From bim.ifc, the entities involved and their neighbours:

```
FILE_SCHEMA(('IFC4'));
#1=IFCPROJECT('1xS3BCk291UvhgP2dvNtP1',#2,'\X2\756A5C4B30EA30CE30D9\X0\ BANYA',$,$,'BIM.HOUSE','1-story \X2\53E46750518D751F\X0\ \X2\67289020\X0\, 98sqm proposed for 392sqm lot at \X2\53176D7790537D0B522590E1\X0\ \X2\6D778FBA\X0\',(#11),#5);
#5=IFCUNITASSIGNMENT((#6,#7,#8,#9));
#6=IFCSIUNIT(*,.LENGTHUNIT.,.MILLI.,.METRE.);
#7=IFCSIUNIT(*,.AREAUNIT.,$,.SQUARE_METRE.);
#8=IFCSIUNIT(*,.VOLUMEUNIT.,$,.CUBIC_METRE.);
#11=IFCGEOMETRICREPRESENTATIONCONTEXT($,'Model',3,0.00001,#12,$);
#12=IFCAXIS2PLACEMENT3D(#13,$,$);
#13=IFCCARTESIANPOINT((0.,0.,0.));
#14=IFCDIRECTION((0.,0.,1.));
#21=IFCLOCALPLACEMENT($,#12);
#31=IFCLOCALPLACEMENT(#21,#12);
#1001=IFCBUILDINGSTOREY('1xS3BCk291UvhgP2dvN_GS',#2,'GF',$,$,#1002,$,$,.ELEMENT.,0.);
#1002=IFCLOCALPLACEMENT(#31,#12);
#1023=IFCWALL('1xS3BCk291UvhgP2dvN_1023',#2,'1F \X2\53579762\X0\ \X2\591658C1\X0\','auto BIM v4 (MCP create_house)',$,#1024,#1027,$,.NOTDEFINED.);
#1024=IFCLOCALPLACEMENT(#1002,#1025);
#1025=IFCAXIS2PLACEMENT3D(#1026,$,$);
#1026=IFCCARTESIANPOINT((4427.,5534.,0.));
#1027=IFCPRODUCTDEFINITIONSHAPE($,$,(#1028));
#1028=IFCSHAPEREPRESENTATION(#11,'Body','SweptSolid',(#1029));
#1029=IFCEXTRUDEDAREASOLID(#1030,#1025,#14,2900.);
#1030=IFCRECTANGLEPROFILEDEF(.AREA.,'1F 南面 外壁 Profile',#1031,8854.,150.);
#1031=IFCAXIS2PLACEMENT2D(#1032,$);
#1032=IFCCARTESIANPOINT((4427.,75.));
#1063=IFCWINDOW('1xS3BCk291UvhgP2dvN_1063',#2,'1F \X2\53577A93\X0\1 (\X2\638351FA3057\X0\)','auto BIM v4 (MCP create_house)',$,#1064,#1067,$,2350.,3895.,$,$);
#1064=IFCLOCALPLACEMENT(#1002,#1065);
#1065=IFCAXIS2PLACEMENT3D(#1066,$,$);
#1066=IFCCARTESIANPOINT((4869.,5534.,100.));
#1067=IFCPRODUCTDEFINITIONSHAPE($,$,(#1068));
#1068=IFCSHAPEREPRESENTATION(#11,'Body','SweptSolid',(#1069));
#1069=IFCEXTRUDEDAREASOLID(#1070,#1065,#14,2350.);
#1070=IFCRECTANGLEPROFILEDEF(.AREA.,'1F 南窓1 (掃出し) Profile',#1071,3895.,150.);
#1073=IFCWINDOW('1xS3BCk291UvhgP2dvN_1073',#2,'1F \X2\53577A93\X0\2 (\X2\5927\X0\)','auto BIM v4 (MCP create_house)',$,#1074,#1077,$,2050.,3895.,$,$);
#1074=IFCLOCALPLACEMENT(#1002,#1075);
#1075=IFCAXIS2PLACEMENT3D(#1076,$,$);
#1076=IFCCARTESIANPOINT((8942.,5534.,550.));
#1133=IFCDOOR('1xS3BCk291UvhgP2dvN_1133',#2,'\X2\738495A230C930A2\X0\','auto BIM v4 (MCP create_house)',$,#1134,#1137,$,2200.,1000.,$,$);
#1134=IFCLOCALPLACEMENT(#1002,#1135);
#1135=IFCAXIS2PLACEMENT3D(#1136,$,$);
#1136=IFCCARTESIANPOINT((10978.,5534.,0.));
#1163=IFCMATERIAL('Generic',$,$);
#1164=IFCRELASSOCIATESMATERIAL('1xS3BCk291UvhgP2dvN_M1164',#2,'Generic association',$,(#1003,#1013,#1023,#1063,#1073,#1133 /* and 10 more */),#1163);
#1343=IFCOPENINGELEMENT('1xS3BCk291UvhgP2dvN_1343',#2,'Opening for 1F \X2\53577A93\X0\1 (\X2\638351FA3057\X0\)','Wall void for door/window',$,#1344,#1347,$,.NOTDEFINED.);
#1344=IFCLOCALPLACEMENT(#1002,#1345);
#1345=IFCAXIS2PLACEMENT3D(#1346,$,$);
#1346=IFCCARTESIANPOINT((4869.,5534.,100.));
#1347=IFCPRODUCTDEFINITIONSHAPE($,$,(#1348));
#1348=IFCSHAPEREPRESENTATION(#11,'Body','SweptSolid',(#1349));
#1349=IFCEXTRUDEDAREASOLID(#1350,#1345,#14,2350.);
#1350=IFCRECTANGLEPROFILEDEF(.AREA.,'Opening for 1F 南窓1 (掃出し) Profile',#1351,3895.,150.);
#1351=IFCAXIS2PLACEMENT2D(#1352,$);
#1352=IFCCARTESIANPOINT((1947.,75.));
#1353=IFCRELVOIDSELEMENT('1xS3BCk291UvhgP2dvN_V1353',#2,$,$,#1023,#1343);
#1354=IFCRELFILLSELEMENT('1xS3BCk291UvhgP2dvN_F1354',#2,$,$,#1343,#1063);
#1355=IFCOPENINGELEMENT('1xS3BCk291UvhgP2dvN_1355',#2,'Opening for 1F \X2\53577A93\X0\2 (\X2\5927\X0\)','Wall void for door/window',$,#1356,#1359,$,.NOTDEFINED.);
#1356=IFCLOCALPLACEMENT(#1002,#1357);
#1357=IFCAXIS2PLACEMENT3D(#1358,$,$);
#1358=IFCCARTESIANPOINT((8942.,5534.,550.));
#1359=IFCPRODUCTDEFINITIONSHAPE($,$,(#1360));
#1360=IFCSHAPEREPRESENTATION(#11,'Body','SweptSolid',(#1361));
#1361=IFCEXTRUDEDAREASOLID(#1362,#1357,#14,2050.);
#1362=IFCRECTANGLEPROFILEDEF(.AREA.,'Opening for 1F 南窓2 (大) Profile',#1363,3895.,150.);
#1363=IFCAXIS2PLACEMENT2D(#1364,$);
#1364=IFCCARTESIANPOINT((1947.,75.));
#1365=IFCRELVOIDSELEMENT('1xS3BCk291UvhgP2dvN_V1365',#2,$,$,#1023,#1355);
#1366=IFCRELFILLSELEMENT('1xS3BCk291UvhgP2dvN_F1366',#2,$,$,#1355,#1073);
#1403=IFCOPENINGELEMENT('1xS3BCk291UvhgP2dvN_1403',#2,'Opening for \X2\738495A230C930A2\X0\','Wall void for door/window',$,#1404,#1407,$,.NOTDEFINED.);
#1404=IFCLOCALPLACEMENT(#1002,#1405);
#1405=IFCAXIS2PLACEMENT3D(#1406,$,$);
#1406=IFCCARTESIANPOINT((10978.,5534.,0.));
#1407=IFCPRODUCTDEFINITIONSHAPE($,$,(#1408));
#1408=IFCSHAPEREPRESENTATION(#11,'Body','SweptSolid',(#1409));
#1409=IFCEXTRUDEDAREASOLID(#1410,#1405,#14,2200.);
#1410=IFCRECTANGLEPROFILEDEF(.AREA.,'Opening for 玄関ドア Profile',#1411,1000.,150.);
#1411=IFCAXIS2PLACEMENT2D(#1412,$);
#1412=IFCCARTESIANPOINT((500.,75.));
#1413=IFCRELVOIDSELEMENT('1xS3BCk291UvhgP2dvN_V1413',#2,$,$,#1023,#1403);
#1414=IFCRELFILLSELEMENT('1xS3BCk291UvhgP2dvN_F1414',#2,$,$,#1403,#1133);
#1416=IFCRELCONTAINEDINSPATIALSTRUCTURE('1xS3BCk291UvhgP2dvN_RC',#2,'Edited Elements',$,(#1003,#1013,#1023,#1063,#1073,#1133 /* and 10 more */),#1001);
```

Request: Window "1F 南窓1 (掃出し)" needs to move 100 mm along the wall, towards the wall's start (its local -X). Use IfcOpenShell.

```python
import ifcopenshell
import ifcopenshell.api.geometry
import ifcopenshell.util.placement
import ifcopenshell.util.unit

model = ifcopenshell.open("bim.ifc")
unit_scale = ifcopenshell.util.unit.calculate_unit_scale(model)

window = model.by_guid("1xS3BCk291UvhgP2dvN_1063")
opening = window.FillsVoids[0].RelatingOpeningElement
wall = opening.VoidsElements[0].RelatingBuildingElement

wall_matrix = ifcopenshell.util.placement.get_local_placement(wall.ObjectPlacement)
shift = wall_matrix[:3, 0] * -0.1 / unit_scale
before = ifcopenshell.util.placement.get_local_placement(window.ObjectPlacement)[:3, 3].copy()

# The window is not placed relative to its opening, so move both.
for product in (opening, window):
    matrix = ifcopenshell.util.placement.get_local_placement(product.ObjectPlacement)
    matrix[:3, 3] += shift
    ifcopenshell.api.geometry.edit_object_placement(model, product=product, matrix=matrix, is_si=False)

after = ifcopenshell.util.placement.get_local_placement(window.ObjectPlacement)[:3, 3]
print("window moved by", (after - before).round(3) + 0.0)

model.write("bim-out.ifc")
```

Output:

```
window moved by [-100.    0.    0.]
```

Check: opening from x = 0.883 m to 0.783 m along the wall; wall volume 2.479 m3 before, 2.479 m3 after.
